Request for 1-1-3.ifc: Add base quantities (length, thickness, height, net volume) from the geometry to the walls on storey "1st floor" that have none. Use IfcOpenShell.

First a look at what the model holds.

```python
import ifcopenshell
import ifcopenshell.util.element
import ifcopenshell.util.unit

model = ifcopenshell.open("1-1-3.ifc")
print(model.schema)
for unit_type in ("LENGTHUNIT", "AREAUNIT", "VOLUMEUNIT"):
    print(unit_type, ifcopenshell.util.unit.calculate_unit_scale(model, unit_type))
storey = next(s for s in model.by_type("IfcBuildingStorey") if s.Name == "1st floor")
walls = [e for e in ifcopenshell.util.element.get_decomposition(storey) if e.is_a("IfcWall")]
for e in sorted(walls, key=lambda e: e.id()):
    print(e.id(), e.is_a(), e.Name, list(ifcopenshell.util.element.get_psets(e, qtos_only=True)), sep=" | ")
```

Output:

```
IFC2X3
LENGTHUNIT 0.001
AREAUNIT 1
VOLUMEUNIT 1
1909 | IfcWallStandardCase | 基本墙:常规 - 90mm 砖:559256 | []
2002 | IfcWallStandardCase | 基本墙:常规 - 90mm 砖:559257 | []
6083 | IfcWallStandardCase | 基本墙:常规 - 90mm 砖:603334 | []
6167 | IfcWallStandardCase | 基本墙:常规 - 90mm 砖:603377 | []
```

```python
import ifcopenshell
import ifcopenshell.api.pset
import ifcopenshell.geom
import ifcopenshell.util.element
import ifcopenshell.util.shape
import ifcopenshell.util.unit

model = ifcopenshell.open("1-1-3.ifc")
unit_scale = ifcopenshell.util.unit.calculate_unit_scale(model)
volume_scale = ifcopenshell.util.unit.calculate_unit_scale(model, "VOLUMEUNIT")
settings = ifcopenshell.geom.settings()

storey = next(s for s in model.by_type("IfcBuildingStorey") if s.Name == "1st floor")
walls = [e for e in ifcopenshell.util.element.get_decomposition(storey) if e.is_a("IfcWall")]

for e in sorted(walls, key=lambda e: e.id()):
    if ifcopenshell.util.element.get_psets(e, qtos_only=True, should_inherit=False):
        continue
    # Geometry comes back in metres, in the element's own axes.
    shape = ifcopenshell.geom.create_shape(settings, e)
    values = {
        "Length": ifcopenshell.util.shape.get_x(shape.geometry) / unit_scale,
        "Width": ifcopenshell.util.shape.get_y(shape.geometry) / unit_scale,
        "Height": ifcopenshell.util.shape.get_z(shape.geometry) / unit_scale,
        "NetVolume": ifcopenshell.util.shape.get_volume(shape.geometry) / volume_scale,
    }
    qto = ifcopenshell.api.pset.add_qto(model, product=e, name="BaseQuantities")
    ifcopenshell.api.pset.edit_qto(model, qto=qto, properties=values)
    print(e.id(), {k: round(v, 3) for k, v in values.items()})

model.write("1-1-3-out.ifc")
```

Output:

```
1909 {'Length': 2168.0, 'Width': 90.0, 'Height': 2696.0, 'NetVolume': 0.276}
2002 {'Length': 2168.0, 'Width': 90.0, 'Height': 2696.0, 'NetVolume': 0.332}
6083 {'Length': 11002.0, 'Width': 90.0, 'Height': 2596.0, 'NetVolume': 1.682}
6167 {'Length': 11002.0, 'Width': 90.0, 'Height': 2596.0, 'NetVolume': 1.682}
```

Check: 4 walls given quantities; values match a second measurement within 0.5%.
